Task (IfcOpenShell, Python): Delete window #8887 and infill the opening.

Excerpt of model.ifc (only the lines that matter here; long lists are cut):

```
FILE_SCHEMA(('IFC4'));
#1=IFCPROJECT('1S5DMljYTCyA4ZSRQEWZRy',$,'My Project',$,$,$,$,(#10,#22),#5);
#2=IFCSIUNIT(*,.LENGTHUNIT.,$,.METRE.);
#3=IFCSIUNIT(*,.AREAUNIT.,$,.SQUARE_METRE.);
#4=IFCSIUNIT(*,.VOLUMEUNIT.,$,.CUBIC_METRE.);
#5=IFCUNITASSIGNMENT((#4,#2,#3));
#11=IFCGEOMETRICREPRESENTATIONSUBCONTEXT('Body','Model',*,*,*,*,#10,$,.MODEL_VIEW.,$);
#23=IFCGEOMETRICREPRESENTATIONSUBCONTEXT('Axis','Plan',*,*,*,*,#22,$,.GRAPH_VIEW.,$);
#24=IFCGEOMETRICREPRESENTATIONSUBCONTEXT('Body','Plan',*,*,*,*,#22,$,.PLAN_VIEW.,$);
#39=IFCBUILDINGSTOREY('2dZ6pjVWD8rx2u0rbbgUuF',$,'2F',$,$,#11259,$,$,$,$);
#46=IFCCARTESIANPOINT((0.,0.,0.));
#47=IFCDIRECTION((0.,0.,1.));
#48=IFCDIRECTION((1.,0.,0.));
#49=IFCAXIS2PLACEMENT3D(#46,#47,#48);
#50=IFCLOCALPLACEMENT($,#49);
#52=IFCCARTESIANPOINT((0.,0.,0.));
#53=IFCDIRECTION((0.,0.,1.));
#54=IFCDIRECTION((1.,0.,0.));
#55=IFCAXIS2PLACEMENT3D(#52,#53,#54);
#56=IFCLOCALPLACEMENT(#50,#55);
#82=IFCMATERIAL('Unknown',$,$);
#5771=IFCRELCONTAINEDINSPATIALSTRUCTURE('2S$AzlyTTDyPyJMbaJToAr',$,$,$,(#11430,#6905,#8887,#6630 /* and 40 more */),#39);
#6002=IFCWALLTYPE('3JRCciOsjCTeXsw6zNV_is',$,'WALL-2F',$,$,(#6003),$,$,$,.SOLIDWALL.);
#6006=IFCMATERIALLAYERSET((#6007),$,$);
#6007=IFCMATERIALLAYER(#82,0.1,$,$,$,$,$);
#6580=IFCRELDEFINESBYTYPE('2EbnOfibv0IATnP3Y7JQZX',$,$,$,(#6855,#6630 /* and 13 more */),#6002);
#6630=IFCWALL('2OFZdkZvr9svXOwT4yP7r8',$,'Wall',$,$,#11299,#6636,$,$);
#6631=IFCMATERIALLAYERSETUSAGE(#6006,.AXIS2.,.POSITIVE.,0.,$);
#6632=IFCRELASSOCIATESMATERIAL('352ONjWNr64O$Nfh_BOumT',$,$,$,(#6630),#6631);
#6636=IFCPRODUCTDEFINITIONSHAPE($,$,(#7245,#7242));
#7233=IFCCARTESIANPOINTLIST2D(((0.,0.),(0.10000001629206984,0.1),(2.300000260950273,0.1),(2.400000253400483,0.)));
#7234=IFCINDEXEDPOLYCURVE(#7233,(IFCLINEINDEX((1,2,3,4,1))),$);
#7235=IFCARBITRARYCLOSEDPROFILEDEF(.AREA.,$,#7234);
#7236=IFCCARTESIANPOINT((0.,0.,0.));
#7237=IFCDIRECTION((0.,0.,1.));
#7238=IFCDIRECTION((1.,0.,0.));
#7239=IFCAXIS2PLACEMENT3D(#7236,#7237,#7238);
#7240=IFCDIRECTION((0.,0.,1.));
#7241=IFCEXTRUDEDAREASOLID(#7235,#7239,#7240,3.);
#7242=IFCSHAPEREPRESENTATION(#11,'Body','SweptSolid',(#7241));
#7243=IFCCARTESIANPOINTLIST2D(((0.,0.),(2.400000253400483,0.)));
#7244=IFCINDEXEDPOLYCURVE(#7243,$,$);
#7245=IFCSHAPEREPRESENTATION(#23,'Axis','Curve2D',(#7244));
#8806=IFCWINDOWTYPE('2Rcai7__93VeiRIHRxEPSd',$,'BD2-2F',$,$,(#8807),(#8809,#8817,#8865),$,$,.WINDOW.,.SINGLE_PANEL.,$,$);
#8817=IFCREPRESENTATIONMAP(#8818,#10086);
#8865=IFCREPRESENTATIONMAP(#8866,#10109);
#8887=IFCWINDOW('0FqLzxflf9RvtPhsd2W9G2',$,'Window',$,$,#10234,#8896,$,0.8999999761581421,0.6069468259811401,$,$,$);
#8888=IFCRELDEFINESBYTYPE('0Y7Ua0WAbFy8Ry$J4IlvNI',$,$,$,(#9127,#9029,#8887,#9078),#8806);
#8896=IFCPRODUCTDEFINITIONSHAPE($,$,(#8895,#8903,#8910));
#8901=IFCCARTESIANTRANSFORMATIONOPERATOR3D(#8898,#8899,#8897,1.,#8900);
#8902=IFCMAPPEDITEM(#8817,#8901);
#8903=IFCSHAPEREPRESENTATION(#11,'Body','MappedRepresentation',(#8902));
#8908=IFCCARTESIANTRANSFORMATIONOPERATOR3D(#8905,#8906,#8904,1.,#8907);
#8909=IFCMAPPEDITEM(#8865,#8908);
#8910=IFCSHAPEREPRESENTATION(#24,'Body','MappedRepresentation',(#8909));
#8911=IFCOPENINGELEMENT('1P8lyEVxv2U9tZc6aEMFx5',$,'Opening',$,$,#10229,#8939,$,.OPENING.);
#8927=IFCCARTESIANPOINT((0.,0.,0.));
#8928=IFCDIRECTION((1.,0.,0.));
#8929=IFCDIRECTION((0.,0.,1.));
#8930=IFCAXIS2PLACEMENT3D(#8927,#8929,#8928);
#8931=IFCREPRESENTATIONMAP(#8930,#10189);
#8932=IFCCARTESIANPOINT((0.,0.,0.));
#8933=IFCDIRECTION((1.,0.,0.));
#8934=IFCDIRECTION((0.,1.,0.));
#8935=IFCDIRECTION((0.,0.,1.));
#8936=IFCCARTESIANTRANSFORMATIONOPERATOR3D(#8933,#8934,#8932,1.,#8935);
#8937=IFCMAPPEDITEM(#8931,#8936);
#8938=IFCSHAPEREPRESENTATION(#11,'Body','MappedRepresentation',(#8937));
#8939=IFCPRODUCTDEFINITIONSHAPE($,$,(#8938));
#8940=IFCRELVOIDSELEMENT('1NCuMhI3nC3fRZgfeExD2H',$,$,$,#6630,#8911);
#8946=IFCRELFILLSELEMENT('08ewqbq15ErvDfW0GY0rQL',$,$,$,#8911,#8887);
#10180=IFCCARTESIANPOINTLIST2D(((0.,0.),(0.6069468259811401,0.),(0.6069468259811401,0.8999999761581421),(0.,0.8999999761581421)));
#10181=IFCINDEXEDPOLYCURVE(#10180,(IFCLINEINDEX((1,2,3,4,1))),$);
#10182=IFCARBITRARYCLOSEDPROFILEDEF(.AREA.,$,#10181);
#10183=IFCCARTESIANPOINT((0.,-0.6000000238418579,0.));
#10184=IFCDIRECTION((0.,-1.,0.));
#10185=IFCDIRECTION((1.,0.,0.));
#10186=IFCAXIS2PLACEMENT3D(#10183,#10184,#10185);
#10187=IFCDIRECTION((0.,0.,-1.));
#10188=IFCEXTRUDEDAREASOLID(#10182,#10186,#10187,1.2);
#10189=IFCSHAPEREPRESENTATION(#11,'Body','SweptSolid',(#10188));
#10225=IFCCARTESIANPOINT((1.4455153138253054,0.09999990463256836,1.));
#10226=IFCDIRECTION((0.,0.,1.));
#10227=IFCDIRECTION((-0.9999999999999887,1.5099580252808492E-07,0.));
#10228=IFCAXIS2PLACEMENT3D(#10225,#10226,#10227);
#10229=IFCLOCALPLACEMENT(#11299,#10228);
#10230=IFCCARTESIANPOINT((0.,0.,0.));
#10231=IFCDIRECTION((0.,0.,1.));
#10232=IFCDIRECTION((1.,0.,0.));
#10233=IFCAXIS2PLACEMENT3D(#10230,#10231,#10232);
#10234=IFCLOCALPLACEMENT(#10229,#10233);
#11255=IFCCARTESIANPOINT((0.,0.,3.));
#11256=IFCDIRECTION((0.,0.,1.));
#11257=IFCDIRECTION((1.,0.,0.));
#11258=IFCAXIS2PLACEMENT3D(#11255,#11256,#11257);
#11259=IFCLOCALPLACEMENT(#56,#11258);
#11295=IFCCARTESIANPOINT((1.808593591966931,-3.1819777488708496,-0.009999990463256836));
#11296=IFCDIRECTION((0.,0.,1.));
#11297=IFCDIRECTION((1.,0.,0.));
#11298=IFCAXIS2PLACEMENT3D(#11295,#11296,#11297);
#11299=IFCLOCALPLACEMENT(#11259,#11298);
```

```python
import ifcopenshell
import ifcopenshell.api.feature
import ifcopenshell.api.root
import ifcopenshell.geom
import ifcopenshell.util.shape

model = ifcopenshell.open("model.ifc")
settings = ifcopenshell.geom.settings()


def volume(element):
    """Net volume in cubic metres, openings subtracted."""
    shape = ifcopenshell.geom.create_shape(settings, element)
    return ifcopenshell.util.shape.get_volume(shape.geometry)


window = model.by_guid("0FqLzxflf9RvtPhsd2W9G2")
opening = window.FillsVoids[0].RelatingOpeningElement
wall = opening.VoidsElements[0].RelatingBuildingElement
before = volume(wall)

ifcopenshell.api.root.remove_product(model, product=window)
ifcopenshell.api.feature.remove_feature(model, feature=opening)

after = volume(wall)

print(f"wall volume {before:.3f} -> {after:.3f} m3")

model.write("model_updated.ifc")
```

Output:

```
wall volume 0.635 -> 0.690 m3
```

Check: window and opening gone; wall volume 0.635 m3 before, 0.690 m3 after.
